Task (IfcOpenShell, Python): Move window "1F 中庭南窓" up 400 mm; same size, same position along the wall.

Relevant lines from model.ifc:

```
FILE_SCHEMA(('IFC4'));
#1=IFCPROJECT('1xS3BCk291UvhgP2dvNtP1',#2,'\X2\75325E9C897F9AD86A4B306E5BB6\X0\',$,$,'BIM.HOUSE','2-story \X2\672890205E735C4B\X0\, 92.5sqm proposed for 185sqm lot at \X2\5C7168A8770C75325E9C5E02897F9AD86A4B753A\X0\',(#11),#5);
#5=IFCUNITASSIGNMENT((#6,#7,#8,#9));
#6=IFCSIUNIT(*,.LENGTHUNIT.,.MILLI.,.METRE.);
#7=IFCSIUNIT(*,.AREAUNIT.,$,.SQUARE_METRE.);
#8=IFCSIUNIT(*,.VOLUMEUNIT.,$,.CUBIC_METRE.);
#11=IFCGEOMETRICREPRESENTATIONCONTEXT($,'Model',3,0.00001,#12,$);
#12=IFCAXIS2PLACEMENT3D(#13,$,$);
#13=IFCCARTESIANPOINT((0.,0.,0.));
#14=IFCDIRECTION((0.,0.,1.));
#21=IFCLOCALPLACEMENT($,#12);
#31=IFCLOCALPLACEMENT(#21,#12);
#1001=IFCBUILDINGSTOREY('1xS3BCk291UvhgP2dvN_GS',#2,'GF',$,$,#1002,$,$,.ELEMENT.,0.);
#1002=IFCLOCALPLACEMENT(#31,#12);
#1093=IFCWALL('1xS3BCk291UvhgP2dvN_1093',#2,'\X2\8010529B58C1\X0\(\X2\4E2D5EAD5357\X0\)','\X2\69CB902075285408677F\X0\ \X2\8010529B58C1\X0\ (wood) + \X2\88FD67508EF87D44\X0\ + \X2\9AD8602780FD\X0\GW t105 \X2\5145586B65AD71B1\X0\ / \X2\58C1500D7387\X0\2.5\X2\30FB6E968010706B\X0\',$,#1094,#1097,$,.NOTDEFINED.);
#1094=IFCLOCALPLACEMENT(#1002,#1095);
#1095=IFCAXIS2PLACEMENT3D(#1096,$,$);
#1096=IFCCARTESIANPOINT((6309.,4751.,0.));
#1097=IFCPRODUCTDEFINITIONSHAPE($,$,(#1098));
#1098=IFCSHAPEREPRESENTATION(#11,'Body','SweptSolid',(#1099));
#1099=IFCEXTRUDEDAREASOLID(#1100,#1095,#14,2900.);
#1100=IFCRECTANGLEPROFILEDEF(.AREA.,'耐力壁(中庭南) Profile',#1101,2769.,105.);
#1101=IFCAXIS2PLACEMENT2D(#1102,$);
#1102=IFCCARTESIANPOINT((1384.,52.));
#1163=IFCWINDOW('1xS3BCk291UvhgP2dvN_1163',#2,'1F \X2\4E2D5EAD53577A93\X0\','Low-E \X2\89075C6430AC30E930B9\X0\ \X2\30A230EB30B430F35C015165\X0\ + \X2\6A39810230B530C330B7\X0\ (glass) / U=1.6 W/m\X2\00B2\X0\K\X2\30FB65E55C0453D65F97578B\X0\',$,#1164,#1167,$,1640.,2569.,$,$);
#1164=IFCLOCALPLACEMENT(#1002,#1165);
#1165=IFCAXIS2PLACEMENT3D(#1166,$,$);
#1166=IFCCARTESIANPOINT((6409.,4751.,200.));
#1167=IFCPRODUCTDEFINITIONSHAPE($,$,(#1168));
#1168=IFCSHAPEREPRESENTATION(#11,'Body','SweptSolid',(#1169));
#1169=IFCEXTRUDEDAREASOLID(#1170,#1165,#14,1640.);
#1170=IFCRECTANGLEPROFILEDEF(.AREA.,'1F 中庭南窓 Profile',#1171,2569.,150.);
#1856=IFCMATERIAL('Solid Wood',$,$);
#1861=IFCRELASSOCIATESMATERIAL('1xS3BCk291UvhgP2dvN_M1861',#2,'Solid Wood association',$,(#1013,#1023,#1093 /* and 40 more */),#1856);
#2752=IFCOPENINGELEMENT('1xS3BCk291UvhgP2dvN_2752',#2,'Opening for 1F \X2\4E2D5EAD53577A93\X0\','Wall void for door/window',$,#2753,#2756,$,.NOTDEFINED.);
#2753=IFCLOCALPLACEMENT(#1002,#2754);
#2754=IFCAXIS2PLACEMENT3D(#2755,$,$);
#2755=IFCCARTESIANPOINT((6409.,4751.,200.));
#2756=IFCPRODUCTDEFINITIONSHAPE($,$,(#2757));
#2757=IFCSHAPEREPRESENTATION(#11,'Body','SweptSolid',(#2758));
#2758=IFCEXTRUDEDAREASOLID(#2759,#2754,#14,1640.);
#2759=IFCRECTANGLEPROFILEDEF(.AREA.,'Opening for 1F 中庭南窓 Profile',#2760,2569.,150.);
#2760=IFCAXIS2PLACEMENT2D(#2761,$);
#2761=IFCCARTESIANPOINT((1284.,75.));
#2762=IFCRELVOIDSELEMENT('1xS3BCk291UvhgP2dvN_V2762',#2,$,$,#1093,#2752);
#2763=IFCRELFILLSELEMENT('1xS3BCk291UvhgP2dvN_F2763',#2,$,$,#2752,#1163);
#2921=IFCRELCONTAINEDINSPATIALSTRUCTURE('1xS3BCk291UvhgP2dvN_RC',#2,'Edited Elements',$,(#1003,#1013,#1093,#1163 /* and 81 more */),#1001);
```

```python
import numpy as np
import ifcopenshell
import ifcopenshell.api.geometry
import ifcopenshell.util.placement
import ifcopenshell.util.unit

model = ifcopenshell.open("model.ifc")
unit_scale = ifcopenshell.util.unit.calculate_unit_scale(model)

window = model.by_id(1163)
opening = window.FillsVoids[0].RelatingOpeningElement
dz = 0.4 / unit_scale

shift = np.array([0.0, 0.0, dz])
# The window is not placed relative to its opening, so move both.
for product in (opening, window):
    matrix = ifcopenshell.util.placement.get_local_placement(product.ObjectPlacement)
    matrix[:3, 3] += shift
    ifcopenshell.api.geometry.edit_object_placement(model, product=product, matrix=matrix, is_si=False)

print(f"moved by {dz * unit_scale:+.3f} m")

model.write("model_updated.ifc")
```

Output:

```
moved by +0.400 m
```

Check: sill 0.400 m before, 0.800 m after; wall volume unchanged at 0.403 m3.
